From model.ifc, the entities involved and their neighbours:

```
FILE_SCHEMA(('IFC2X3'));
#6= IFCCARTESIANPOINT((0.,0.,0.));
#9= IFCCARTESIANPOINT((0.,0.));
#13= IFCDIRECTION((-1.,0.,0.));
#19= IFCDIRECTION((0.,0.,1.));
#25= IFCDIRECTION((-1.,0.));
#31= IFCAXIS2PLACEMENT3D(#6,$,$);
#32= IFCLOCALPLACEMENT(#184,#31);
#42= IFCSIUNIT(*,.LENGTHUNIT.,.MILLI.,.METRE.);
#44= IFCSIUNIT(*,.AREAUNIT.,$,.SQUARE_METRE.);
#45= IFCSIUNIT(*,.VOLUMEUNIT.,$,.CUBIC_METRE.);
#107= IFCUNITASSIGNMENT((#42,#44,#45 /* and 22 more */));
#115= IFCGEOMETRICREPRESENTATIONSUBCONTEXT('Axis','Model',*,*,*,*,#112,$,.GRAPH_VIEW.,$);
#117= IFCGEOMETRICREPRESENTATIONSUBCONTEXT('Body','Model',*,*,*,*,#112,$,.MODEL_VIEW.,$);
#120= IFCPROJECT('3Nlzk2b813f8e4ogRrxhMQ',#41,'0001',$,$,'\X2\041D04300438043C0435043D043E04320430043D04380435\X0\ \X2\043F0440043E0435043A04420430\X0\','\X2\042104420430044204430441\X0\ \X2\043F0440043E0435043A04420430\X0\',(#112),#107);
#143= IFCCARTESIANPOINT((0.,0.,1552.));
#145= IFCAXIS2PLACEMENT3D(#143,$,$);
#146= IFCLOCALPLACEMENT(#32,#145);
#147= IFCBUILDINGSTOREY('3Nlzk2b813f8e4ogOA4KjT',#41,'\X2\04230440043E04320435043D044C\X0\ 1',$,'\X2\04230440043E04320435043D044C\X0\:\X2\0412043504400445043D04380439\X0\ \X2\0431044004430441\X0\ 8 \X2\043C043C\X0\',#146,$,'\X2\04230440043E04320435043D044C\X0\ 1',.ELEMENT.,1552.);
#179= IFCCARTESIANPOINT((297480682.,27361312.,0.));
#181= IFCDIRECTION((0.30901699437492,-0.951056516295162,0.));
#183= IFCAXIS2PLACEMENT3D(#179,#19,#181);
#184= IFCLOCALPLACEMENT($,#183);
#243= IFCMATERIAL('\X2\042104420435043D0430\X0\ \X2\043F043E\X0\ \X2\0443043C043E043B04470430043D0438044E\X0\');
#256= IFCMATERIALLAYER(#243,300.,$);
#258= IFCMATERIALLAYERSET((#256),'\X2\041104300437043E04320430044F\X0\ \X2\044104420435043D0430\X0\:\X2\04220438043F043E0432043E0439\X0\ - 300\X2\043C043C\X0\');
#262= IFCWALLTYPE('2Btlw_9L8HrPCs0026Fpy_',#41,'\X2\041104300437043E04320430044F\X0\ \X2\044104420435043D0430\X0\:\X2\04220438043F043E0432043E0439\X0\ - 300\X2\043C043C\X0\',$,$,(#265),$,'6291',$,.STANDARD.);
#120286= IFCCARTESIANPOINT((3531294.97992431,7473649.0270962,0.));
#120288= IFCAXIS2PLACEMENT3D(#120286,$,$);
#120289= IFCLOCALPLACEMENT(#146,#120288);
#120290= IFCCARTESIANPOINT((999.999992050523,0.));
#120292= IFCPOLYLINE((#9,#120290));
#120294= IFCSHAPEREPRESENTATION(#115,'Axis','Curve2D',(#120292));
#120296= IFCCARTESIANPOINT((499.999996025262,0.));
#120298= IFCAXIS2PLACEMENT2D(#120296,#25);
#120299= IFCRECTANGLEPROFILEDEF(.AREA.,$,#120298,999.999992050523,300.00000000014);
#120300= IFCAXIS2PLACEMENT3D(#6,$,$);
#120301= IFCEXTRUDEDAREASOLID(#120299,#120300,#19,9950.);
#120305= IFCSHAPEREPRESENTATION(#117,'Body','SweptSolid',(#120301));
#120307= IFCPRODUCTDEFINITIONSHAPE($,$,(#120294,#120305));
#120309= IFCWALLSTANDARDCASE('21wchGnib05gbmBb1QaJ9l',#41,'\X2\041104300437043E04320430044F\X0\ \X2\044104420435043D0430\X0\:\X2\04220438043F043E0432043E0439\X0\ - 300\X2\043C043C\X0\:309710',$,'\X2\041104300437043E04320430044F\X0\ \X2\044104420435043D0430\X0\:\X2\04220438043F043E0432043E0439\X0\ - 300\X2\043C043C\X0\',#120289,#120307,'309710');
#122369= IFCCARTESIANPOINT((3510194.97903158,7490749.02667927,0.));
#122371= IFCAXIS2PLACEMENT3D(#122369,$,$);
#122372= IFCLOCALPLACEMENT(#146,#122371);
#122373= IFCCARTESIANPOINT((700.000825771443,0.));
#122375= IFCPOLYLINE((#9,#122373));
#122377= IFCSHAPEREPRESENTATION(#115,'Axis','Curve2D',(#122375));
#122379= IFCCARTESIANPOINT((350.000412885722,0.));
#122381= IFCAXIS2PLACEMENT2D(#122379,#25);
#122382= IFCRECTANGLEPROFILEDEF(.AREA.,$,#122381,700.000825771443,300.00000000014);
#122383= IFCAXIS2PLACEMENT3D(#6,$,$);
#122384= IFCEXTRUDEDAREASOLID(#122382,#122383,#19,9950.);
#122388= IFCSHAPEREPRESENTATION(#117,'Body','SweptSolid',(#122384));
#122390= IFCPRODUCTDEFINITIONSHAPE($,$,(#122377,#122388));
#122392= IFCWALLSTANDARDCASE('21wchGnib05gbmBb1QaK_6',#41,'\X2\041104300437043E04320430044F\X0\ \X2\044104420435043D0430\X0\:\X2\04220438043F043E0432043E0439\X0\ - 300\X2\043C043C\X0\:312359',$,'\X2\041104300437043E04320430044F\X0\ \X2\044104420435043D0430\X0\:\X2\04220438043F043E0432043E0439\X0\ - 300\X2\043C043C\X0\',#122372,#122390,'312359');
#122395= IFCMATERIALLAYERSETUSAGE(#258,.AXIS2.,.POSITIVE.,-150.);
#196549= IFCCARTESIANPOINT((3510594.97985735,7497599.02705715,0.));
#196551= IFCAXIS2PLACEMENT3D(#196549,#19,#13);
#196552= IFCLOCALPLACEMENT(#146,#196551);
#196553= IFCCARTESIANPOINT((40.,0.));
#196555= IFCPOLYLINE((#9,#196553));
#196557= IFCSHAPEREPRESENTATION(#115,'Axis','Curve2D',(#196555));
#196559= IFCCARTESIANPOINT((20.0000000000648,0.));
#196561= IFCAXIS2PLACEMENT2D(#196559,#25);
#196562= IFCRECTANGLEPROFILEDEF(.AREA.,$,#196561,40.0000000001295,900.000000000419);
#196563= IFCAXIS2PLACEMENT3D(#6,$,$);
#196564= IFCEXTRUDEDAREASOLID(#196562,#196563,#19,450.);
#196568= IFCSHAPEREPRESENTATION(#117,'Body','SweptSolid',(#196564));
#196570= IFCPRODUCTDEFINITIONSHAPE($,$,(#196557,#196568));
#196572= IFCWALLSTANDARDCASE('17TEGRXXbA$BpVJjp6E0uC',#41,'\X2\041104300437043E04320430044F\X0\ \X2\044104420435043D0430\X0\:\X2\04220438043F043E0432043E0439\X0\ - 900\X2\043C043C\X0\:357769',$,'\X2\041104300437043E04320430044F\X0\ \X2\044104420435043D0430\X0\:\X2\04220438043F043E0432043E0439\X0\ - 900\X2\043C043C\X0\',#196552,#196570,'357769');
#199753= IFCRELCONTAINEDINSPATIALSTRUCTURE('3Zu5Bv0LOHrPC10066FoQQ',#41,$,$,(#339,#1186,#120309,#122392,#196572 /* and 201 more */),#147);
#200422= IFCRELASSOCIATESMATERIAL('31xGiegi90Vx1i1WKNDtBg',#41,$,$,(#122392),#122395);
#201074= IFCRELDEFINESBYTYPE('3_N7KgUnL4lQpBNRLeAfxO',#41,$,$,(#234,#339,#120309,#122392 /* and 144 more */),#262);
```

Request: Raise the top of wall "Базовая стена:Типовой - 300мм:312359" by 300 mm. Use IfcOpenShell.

```python
import ifcopenshell
import ifcopenshell.geom
import ifcopenshell.util.representation
import ifcopenshell.util.shape
import ifcopenshell.util.unit

model = ifcopenshell.open("model.ifc")
unit_scale = ifcopenshell.util.unit.calculate_unit_scale(model)
settings = ifcopenshell.geom.settings()


def volume(element):
    """Net volume in cubic metres, openings subtracted."""
    shape = ifcopenshell.geom.create_shape(settings, element)
    return ifcopenshell.util.shape.get_volume(shape.geometry)


wall = model.by_id(122392)
before = volume(wall)

body = ifcopenshell.util.representation.get_representation(wall, "Model", "Body")
solid = body.Items[0]
old_height = solid.Depth
solid.Depth += 0.3 / unit_scale
after = volume(wall)

print(f"height {old_height:g} -> {solid.Depth:g}, volume {before:.3f} -> {after:.3f} m3")

model.write("model_rev.ifc")
```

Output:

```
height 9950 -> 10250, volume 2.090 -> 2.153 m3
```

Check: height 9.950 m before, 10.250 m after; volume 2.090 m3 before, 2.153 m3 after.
